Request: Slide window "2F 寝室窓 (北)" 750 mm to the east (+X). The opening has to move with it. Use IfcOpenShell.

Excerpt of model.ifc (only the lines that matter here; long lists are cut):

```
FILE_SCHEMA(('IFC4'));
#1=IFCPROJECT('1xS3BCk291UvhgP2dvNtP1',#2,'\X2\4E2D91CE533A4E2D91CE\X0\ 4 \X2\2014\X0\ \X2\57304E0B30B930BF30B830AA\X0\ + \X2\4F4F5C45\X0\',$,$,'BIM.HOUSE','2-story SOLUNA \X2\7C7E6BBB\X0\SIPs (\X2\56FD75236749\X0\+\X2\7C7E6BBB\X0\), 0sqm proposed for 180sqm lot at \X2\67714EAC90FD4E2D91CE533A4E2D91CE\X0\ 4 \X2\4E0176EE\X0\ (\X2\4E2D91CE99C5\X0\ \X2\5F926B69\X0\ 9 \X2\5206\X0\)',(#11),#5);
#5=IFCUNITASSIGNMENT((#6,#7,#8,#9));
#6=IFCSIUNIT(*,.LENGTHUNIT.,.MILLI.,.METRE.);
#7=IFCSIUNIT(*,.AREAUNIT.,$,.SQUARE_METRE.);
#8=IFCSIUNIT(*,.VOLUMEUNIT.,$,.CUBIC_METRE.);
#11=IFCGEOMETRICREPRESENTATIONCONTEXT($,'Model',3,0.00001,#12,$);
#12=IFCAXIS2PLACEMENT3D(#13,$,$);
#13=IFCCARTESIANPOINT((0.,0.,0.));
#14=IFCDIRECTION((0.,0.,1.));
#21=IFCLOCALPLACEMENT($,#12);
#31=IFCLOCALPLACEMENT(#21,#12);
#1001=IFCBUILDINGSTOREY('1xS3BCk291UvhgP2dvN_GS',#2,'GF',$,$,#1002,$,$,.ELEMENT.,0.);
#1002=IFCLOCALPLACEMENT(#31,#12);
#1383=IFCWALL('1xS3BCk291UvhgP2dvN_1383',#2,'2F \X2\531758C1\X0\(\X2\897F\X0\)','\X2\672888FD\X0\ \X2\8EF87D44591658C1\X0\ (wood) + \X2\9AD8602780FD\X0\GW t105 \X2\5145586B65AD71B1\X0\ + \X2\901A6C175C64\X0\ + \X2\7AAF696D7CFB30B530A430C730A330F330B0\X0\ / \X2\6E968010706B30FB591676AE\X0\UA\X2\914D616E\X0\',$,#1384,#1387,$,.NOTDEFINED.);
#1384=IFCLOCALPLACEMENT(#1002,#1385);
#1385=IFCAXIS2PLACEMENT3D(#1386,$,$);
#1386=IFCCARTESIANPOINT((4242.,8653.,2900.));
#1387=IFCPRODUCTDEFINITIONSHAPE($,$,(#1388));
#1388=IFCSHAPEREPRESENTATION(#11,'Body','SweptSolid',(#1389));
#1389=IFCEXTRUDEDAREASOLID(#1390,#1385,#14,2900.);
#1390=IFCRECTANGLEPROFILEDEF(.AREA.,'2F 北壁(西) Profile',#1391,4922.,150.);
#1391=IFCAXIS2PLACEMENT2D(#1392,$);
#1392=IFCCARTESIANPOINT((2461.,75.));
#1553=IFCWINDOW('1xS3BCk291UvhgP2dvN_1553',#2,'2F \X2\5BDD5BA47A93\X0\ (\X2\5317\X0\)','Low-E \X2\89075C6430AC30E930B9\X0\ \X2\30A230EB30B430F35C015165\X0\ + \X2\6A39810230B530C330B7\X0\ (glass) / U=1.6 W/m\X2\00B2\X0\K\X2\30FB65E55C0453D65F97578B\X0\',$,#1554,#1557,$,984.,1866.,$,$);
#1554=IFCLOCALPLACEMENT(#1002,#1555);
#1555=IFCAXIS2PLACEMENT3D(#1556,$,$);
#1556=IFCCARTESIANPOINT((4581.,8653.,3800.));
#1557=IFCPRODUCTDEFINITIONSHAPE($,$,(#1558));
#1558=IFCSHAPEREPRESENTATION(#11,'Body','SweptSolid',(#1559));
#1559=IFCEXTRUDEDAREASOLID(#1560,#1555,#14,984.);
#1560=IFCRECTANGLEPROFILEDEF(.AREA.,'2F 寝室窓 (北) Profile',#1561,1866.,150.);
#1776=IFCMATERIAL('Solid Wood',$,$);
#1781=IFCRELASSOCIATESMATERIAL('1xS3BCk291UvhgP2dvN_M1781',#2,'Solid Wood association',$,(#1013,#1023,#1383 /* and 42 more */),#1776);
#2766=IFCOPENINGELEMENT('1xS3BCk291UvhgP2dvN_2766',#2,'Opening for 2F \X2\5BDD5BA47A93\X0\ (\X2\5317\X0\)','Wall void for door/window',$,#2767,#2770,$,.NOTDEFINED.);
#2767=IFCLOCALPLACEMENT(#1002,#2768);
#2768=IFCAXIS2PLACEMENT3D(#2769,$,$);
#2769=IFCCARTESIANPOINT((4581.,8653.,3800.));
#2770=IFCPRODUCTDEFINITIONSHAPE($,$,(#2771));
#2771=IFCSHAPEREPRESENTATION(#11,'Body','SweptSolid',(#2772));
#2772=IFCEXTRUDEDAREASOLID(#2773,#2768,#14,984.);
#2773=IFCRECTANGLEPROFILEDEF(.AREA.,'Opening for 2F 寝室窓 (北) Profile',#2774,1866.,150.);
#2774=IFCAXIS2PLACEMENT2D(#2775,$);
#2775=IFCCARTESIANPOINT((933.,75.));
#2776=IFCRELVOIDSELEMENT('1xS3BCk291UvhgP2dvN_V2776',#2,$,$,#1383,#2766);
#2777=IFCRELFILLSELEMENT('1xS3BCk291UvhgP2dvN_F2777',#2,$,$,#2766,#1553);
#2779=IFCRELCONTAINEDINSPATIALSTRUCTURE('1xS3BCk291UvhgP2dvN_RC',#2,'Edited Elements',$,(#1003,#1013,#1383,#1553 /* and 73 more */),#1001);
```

```python
import ifcopenshell
import ifcopenshell.api.geometry
import ifcopenshell.util.placement
import ifcopenshell.util.unit

model = ifcopenshell.open("model.ifc")
unit_scale = ifcopenshell.util.unit.calculate_unit_scale(model)

window = model.by_guid("1xS3BCk291UvhgP2dvN_1553")
opening = window.FillsVoids[0].RelatingOpeningElement
wall = opening.VoidsElements[0].RelatingBuildingElement

wall_matrix = ifcopenshell.util.placement.get_local_placement(wall.ObjectPlacement)
shift = wall_matrix[:3, 0] * 0.75 / unit_scale
before = ifcopenshell.util.placement.get_local_placement(window.ObjectPlacement)[:3, 3].copy()

# The window is not placed relative to its opening, so move both.
for product in (opening, window):
    matrix = ifcopenshell.util.placement.get_local_placement(product.ObjectPlacement)
    matrix[:3, 3] += shift
    ifcopenshell.api.geometry.edit_object_placement(model, product=product, matrix=matrix, is_si=False)

after = ifcopenshell.util.placement.get_local_placement(window.ObjectPlacement)[:3, 3]
print("window moved by", (after - before).round(3) + 0.0)

model.write("model_edited.ifc")
```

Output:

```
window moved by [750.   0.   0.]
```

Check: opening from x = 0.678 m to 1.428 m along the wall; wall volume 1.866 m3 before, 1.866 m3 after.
